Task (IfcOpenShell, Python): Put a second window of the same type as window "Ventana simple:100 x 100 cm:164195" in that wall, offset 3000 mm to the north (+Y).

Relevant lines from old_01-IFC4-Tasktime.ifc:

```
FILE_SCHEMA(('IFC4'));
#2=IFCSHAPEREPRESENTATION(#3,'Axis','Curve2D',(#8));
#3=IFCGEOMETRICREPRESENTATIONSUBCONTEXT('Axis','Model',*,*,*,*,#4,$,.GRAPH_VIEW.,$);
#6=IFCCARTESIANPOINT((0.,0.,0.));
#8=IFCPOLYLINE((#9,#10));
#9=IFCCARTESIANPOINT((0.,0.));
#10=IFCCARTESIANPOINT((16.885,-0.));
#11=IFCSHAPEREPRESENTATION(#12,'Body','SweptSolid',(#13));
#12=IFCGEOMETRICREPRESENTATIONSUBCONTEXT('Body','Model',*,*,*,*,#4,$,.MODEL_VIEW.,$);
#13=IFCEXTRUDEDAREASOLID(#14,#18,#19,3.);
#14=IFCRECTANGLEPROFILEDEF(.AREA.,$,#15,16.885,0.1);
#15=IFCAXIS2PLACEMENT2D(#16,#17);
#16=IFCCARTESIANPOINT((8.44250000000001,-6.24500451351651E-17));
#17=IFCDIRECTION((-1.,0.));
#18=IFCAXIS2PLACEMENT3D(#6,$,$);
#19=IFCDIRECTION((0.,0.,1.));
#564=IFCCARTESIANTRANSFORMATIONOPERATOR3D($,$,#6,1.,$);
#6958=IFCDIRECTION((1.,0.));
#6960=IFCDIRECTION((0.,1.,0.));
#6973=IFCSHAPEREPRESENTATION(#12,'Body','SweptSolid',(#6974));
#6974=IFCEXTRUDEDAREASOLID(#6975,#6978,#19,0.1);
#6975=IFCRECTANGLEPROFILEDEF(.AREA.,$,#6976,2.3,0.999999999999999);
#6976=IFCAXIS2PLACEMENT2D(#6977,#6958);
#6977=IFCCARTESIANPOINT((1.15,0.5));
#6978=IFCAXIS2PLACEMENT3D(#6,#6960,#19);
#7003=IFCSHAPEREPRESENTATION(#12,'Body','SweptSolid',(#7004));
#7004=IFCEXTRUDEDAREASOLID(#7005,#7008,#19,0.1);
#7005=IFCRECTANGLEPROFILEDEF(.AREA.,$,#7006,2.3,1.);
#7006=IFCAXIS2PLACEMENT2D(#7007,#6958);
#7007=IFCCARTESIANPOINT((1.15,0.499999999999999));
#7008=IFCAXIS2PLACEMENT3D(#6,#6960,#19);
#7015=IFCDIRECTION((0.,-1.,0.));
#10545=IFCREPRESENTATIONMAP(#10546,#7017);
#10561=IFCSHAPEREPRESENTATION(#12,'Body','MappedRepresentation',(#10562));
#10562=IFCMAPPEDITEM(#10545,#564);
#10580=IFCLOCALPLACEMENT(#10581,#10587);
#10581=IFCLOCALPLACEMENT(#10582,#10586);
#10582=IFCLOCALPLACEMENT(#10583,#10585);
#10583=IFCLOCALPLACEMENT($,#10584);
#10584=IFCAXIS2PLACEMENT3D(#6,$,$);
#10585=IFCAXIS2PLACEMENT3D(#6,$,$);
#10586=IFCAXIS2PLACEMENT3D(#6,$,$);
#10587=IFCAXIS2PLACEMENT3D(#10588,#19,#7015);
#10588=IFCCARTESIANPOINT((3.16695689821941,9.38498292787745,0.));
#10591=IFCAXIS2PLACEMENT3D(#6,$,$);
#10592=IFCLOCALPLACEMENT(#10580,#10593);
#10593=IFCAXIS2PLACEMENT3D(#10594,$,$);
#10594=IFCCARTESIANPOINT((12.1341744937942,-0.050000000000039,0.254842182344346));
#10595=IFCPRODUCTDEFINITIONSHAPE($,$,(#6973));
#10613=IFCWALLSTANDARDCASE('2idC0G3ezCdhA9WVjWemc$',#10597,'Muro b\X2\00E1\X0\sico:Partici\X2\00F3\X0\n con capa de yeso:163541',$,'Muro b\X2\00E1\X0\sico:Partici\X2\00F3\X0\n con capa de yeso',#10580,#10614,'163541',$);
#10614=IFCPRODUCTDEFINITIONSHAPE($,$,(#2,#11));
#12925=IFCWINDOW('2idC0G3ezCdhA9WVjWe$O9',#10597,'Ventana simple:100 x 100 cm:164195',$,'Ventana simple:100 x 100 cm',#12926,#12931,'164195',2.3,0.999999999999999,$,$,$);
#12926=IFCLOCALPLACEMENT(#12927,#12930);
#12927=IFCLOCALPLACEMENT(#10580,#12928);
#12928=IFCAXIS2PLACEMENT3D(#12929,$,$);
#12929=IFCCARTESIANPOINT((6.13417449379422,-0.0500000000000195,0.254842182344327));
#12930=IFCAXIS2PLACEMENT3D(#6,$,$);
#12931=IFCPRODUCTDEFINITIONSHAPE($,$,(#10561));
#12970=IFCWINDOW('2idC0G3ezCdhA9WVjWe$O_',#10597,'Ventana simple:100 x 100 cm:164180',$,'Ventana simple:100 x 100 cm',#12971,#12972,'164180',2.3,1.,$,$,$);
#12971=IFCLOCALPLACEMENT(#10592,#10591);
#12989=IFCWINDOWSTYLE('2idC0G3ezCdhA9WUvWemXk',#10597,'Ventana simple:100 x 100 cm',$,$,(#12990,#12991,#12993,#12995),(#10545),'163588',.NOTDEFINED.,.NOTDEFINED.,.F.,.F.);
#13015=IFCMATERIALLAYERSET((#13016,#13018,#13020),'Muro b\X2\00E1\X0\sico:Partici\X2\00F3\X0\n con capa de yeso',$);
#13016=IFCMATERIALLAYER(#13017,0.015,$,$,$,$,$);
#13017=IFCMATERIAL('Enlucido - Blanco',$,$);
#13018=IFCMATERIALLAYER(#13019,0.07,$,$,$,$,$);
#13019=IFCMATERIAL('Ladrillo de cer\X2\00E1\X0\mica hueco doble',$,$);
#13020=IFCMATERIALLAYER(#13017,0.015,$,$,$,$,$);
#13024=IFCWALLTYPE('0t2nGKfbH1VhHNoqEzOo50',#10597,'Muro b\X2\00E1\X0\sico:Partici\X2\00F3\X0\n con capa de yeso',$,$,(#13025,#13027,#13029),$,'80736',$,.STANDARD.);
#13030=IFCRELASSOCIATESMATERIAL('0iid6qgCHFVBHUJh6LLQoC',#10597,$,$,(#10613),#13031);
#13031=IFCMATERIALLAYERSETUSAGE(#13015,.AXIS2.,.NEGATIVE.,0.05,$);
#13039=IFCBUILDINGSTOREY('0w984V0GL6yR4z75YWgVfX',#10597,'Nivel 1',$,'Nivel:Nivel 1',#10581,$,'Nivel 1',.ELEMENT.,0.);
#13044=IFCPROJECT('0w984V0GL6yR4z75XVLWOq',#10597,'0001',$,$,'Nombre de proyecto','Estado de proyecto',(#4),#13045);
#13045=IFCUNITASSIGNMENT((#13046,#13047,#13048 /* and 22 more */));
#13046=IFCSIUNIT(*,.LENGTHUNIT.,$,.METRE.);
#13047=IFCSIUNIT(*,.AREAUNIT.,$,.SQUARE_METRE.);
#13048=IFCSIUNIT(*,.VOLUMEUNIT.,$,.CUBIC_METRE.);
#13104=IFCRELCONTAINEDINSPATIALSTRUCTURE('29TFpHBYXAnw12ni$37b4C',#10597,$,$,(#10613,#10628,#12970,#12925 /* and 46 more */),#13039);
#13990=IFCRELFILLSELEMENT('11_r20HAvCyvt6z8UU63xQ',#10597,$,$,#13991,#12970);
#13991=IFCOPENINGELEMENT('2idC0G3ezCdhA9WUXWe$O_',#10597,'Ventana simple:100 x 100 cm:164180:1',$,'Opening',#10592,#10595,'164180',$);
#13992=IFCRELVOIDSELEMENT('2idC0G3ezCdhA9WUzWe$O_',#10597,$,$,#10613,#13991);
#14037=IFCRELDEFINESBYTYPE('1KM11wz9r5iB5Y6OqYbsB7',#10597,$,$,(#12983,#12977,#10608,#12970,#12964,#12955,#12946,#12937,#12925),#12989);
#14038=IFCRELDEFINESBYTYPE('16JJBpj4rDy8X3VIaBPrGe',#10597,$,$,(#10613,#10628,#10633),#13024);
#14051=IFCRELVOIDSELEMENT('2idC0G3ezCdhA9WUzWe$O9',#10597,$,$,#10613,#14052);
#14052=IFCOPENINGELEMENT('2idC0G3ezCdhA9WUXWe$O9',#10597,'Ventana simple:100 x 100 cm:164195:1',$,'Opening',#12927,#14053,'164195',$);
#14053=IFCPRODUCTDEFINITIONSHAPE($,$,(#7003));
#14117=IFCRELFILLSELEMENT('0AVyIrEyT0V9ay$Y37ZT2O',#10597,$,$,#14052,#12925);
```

```python
import ifcopenshell
import ifcopenshell.api.feature
import ifcopenshell.api.geometry
import ifcopenshell.api.root
import ifcopenshell.geom
import ifcopenshell.util.element
import ifcopenshell.util.placement
import ifcopenshell.util.shape

model = ifcopenshell.open("old_01-IFC4-Tasktime.ifc")
settings = ifcopenshell.geom.settings()


def volume(element):
    """Net volume in cubic metres, openings subtracted."""
    shape = ifcopenshell.geom.create_shape(settings, element)
    return ifcopenshell.util.shape.get_volume(shape.geometry)


def reuse_history(source, copy):
    """copy_class also copies each property set's owner history, people and application; keep the originals."""
    for rel in copy.IsDefinedBy:
        if rel.is_a("IfcRelDefinesByProperties") and (history := rel.RelatingPropertyDefinition.OwnerHistory):
            rel.RelatingPropertyDefinition.OwnerHistory = source.OwnerHistory
            ifcopenshell.util.element.remove_deep2(model, history)


window = model.by_guid("2idC0G3ezCdhA9WVjWe$O9")
opening = window.FillsVoids[0].RelatingOpeningElement
wall = opening.VoidsElements[0].RelatingBuildingElement
before = volume(wall)
shift = ifcopenshell.util.placement.get_local_placement(wall.ObjectPlacement)[:3, 0] * -3.0

# copy_class copies the void relationship, type, container and properties, but no geometry.
new_opening = ifcopenshell.api.root.copy_class(model, product=opening)
new_opening.Representation = ifcopenshell.util.element.copy_deep(
    model, opening.Representation, exclude=["IfcGeometricRepresentationContext", "IfcRepresentationMap"]
)
new_opening.Name = "Ventana simple:100 x 100 cm"
new_opening.Tag = None
new_window = ifcopenshell.api.root.copy_class(model, product=window)
new_window.Representation = ifcopenshell.util.element.copy_deep(
    model, window.Representation, exclude=["IfcGeometricRepresentationContext", "IfcRepresentationMap"]
)
new_window.Name = "Ventana simple:100 x 100 cm"
new_window.Tag = None
reuse_history(window, new_window)
ifcopenshell.api.feature.add_filling(model, opening=new_opening, element=new_window)

for old, new in ((opening, new_opening), (window, new_window)):
    matrix = ifcopenshell.util.placement.get_local_placement(old.ObjectPlacement)
    matrix[:3, 3] += shift
    ifcopenshell.api.geometry.edit_object_placement(model, product=new, matrix=matrix, is_si=False)

after = volume(wall)

print(f"wall volume {before:.3f} -> {after:.3f} m3")

model.write("old_01-IFC4-Tasktime-out.ifc")
```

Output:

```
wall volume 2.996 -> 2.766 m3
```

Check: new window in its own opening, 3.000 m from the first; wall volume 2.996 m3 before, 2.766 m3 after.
